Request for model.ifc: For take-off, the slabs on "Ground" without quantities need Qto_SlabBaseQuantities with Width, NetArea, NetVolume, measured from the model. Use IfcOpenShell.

First a look at what the model holds.

```python
import ifcopenshell
import ifcopenshell.util.element
import ifcopenshell.util.unit

model = ifcopenshell.open("model.ifc")
print(model.schema)
for unit_type in ("LENGTHUNIT", "AREAUNIT", "VOLUMEUNIT"):
    print(unit_type, ifcopenshell.util.unit.calculate_unit_scale(model, unit_type))
storey = next(s for s in model.by_type("IfcBuildingStorey") if s.Name == "Ground")
slabs = [e for e in ifcopenshell.util.element.get_decomposition(storey) if e.is_a("IfcSlab")]
for e in sorted(slabs, key=lambda e: e.id()):
    print(e.id(), e.is_a(), e.Name, list(ifcopenshell.util.element.get_psets(e, qtos_only=True)), sep=" | ")
```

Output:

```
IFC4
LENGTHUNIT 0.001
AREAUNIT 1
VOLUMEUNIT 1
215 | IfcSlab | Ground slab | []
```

```python
import ifcopenshell
import ifcopenshell.api.pset
import ifcopenshell.geom
import ifcopenshell.util.element
import ifcopenshell.util.shape
import ifcopenshell.util.unit

model = ifcopenshell.open("model.ifc")
unit_scale = ifcopenshell.util.unit.calculate_unit_scale(model)
area_scale = ifcopenshell.util.unit.calculate_unit_scale(model, "AREAUNIT")
volume_scale = ifcopenshell.util.unit.calculate_unit_scale(model, "VOLUMEUNIT")
settings = ifcopenshell.geom.settings()

storey = next(s for s in model.by_type("IfcBuildingStorey") if s.Name == "Ground")
slabs = [e for e in ifcopenshell.util.element.get_decomposition(storey) if e.is_a("IfcSlab")]

for e in sorted(slabs, key=lambda e: e.id()):
    if ifcopenshell.util.element.get_psets(e, qtos_only=True, should_inherit=False):
        continue
    # Geometry comes back in metres, in the element's own axes.
    shape = ifcopenshell.geom.create_shape(settings, e)
    values = {
        "Width": ifcopenshell.util.shape.get_z(shape.geometry) / unit_scale,
        "NetArea": ifcopenshell.util.shape.get_footprint_area(shape.geometry) / area_scale,
        "NetVolume": ifcopenshell.util.shape.get_volume(shape.geometry) / volume_scale,
    }
    qto = ifcopenshell.api.pset.add_qto(model, product=e, name="Qto_SlabBaseQuantities")
    ifcopenshell.api.pset.edit_qto(model, qto=qto, properties=values)
    print(e.id(), {k: round(v, 3) for k, v in values.items()})

model.write("model_updated.ifc")
```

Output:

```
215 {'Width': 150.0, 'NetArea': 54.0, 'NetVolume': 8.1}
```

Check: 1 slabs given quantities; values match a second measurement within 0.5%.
